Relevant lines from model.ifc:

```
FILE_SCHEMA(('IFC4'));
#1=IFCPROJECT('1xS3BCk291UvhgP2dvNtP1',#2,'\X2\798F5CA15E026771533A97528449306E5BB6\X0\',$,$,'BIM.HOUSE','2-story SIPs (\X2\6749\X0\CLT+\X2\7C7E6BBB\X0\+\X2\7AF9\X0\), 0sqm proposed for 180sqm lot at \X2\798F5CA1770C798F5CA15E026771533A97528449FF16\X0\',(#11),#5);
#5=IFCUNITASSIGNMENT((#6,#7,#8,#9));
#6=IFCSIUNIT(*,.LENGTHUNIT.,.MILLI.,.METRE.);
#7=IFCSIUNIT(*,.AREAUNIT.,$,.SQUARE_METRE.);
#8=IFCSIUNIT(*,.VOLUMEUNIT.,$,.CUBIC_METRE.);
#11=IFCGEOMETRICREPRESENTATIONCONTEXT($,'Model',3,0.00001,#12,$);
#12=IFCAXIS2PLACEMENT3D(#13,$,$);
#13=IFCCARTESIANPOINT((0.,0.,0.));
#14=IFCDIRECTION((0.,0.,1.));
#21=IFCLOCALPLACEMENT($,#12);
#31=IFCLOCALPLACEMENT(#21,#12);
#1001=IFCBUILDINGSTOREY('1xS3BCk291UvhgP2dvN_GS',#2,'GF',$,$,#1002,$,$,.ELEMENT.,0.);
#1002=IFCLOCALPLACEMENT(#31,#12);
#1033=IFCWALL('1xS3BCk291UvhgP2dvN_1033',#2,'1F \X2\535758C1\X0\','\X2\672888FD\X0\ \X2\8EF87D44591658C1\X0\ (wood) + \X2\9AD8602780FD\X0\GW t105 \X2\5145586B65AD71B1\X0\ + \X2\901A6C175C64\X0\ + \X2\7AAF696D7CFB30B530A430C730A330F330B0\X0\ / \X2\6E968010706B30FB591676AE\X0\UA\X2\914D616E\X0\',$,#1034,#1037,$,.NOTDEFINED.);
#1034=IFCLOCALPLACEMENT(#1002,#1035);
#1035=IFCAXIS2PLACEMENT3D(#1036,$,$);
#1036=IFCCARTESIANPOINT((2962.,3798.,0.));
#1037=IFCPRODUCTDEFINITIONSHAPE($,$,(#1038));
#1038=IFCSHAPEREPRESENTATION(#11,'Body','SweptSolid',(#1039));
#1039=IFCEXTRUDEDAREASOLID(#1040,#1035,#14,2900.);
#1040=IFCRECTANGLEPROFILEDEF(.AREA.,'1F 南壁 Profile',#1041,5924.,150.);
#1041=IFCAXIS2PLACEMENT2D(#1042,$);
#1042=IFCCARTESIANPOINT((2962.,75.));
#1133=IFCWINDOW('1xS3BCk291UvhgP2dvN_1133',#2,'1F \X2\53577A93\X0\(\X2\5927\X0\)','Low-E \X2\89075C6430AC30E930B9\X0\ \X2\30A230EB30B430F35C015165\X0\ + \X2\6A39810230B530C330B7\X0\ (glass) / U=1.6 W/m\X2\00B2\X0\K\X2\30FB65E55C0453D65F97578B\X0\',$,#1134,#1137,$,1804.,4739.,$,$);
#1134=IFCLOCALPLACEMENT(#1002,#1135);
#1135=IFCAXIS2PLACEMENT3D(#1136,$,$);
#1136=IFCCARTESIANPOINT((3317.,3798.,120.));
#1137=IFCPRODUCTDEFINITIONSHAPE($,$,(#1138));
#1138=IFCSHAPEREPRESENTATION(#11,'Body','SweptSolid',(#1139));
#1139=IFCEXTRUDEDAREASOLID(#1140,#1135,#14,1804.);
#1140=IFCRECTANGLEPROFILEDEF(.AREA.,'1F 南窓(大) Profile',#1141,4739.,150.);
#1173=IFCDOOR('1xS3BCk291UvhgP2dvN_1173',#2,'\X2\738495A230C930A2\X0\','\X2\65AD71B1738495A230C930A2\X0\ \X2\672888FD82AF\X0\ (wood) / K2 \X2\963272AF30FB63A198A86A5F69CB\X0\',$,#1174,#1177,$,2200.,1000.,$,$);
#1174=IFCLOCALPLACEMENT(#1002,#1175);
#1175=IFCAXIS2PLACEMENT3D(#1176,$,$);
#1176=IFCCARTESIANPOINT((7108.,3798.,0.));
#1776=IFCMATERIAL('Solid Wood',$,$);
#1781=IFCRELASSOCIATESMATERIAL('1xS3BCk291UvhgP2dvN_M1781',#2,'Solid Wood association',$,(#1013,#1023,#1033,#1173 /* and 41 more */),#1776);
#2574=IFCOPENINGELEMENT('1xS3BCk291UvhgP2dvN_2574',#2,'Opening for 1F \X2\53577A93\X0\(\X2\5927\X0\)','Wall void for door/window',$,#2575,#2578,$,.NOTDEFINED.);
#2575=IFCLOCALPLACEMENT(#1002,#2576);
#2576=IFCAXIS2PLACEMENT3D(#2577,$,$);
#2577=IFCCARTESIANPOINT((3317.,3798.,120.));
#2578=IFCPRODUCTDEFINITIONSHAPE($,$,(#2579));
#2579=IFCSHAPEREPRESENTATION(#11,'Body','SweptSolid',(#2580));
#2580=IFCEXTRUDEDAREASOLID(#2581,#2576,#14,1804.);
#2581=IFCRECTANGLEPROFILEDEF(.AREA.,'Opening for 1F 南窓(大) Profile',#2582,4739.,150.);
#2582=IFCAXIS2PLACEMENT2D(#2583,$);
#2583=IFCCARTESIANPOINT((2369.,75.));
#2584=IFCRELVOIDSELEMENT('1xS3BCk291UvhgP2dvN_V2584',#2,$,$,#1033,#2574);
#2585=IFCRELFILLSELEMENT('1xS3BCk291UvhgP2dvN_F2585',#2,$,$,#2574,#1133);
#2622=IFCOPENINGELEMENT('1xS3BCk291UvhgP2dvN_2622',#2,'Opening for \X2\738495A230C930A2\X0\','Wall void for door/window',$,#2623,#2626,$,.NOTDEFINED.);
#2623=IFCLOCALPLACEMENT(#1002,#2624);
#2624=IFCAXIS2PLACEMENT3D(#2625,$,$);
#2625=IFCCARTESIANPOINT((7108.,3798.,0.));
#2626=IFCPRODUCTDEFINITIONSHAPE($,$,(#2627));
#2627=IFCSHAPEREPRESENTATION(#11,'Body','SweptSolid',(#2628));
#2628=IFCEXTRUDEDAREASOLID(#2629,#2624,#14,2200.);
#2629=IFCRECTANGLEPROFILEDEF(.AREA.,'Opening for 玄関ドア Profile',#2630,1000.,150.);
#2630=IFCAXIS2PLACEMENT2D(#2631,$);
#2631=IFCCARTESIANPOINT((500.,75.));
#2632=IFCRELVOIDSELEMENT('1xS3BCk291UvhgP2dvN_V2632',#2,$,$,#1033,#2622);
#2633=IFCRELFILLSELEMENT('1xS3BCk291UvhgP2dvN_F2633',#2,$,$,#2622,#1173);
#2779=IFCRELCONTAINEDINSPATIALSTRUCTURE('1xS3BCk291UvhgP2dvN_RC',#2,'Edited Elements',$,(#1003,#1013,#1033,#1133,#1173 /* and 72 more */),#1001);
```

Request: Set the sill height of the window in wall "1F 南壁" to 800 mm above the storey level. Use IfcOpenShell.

```python
import numpy as np
import ifcopenshell
import ifcopenshell.api.geometry
import ifcopenshell.geom
import ifcopenshell.util.element
import ifcopenshell.util.placement
import ifcopenshell.util.shape
import ifcopenshell.util.unit

model = ifcopenshell.open("model.ifc")
unit_scale = ifcopenshell.util.unit.calculate_unit_scale(model)

window = model.by_guid("1xS3BCk291UvhgP2dvN_1133")
opening = window.FillsVoids[0].RelatingOpeningElement
storey = ifcopenshell.util.element.get_container(window, ifc_class="IfcBuildingStorey")
level = ifcopenshell.util.placement.get_local_placement(storey.ObjectPlacement)[2, 3]

# The opening's origin need not be at the sill, so measure its lowest point.
shape = ifcopenshell.geom.create_shape(ifcopenshell.geom.settings(), opening)
bottom = ifcopenshell.util.shape.get_shape_bottom_elevation(shape, shape.geometry) / unit_scale
dz = level + 0.8 / unit_scale - bottom

shift = np.array([0.0, 0.0, dz])
# The window is not placed relative to its opening, so move both.
for product in (opening, window):
    matrix = ifcopenshell.util.placement.get_local_placement(product.ObjectPlacement)
    matrix[:3, 3] += shift
    ifcopenshell.api.geometry.edit_object_placement(model, product=product, matrix=matrix, is_si=False)

print(f"moved by {dz * unit_scale:+.3f} m")

model.write("model_v2.ifc")
```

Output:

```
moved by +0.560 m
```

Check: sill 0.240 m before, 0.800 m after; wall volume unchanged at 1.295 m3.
